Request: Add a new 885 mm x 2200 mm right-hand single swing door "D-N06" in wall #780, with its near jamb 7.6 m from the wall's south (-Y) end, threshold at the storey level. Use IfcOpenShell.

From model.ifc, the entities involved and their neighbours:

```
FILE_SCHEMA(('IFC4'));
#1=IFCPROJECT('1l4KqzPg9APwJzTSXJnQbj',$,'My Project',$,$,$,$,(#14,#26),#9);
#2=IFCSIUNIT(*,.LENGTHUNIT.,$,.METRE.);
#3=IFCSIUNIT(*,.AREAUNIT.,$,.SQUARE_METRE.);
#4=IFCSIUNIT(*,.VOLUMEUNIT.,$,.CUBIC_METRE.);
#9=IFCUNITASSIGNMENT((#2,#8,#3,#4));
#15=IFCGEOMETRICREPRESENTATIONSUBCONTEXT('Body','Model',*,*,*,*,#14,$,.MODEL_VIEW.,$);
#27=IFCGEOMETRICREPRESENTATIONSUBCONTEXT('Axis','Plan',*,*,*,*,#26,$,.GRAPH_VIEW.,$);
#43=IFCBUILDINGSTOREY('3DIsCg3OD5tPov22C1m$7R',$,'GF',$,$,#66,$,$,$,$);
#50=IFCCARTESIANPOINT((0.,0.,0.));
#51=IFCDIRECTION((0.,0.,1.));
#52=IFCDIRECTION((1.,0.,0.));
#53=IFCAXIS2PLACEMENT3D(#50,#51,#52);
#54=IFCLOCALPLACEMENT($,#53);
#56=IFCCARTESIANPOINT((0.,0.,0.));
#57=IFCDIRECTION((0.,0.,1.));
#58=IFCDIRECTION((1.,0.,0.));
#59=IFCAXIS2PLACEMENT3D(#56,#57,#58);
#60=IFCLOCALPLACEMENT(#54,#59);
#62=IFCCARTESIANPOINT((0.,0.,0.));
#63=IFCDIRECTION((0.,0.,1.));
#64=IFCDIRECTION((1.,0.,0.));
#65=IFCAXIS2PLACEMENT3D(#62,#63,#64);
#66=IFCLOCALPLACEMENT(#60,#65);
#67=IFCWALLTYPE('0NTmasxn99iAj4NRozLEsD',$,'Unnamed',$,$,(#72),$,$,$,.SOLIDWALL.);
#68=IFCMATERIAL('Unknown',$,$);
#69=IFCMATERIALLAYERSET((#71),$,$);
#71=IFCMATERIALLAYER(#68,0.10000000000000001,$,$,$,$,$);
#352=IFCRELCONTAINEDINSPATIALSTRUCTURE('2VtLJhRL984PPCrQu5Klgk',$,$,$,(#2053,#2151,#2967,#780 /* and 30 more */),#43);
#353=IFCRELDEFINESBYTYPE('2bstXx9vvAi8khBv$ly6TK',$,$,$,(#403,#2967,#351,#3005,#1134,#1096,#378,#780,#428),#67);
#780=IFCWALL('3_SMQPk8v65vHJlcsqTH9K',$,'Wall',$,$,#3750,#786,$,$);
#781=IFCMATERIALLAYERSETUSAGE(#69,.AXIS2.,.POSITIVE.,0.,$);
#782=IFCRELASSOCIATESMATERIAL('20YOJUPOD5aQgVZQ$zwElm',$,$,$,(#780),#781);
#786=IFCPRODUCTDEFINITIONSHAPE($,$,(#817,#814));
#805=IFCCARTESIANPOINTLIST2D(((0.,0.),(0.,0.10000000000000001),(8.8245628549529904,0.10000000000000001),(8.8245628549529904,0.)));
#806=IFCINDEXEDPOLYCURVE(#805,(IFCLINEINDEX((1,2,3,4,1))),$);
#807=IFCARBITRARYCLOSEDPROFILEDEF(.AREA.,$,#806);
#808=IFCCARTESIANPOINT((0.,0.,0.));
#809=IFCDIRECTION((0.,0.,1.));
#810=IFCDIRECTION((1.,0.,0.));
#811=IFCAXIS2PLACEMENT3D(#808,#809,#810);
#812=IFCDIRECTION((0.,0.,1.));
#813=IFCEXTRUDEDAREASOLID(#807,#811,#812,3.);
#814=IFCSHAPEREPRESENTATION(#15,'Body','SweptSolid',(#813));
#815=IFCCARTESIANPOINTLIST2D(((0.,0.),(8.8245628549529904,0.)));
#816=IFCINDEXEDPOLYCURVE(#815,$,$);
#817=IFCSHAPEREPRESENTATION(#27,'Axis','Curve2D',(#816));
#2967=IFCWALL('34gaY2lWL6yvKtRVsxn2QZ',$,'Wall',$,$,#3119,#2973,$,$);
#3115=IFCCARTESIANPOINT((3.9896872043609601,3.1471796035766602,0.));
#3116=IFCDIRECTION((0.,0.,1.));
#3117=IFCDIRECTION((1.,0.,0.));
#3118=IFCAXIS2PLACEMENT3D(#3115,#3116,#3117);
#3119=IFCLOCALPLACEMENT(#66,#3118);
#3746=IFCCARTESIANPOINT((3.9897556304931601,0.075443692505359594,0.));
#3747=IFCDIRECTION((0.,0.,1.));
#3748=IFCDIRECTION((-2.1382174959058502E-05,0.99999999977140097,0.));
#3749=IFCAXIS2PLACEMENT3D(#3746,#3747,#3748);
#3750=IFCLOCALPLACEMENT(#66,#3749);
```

```python
import numpy as np
import ifcopenshell
import ifcopenshell.api.feature
import ifcopenshell.api.geometry
import ifcopenshell.api.root
import ifcopenshell.api.spatial
import ifcopenshell.geom
import ifcopenshell.util.element
import ifcopenshell.util.placement
import ifcopenshell.util.representation
import ifcopenshell.util.shape
import ifcopenshell.util.unit

model = ifcopenshell.open("model.ifc")
unit_scale = ifcopenshell.util.unit.calculate_unit_scale(model)
settings = ifcopenshell.geom.settings()


def volume(element):
    """Net volume in cubic metres, openings subtracted."""
    shape = ifcopenshell.geom.create_shape(settings, element)
    return ifcopenshell.util.shape.get_volume(shape.geometry)


wall = model.by_guid("3_SMQPk8v65vHJlcsqTH9K")
storey = ifcopenshell.util.element.get_container(wall, ifc_class="IfcBuildingStorey")
context = ifcopenshell.util.representation.get_context(model, "Model", "Body", "MODEL_VIEW")
before = volume(wall)

width, height, from_end, sill = 0.885, 2.2, 7.6, 0.0  # metres

# The wall runs along its own X axis, and the end named is its -X end.
wall_shape = ifcopenshell.geom.create_shape(settings, wall)
x, y, z = ifcopenshell.util.shape.get_vertices(wall_shape.geometry).T
start = x.min() + from_end
face, thickness = float(y.min()), float(y.max() - y.min())
wall_matrix = ifcopenshell.util.placement.get_local_placement(wall.ObjectPlacement)
level = ifcopenshell.util.placement.get_local_placement(storey.ObjectPlacement)[2, 3]


def in_wall(x, y):
    """Placement at x, y metres in the wall's axes, at sill height."""
    matrix = wall_matrix.copy()
    matrix[:, 3] = wall_matrix @ np.array([x / unit_scale, y / unit_scale, 0.0, 1.0])
    matrix[2, 3] = level + sill / unit_scale
    return matrix


# Opening: a box that overshoots both wall faces by 50 mm.
opening = ifcopenshell.api.root.create_entity(model, ifc_class="IfcOpeningElement", predefined_type="OPENING")
box = ifcopenshell.api.geometry.add_wall_representation(
    model, context=context, length=width, height=height, thickness=thickness + 0.1
)
ifcopenshell.api.geometry.assign_representation(model, product=opening, representation=box)
ifcopenshell.api.geometry.edit_object_placement(model, product=opening, matrix=in_wall(start, face - 0.05), is_si=False)
ifcopenshell.api.feature.add_feature(model, feature=opening, element=wall)

door = ifcopenshell.api.root.create_entity(model, ifc_class="IfcDoor", name="D-N06", predefined_type="DOOR")
door.OverallWidth, door.OverallHeight = width / unit_scale, height / unit_scale
door.OperationType = "SINGLE_SWING_RIGHT"
body = ifcopenshell.api.geometry.add_door_representation(
    model,
    context=context,
    overall_width=door.OverallWidth,
    overall_height=door.OverallHeight,
    operation_type="SINGLE_SWING_RIGHT",
    lining_properties={"LiningDepth": thickness / unit_scale, "ThresholdDepth": thickness / unit_scale},
)
ifcopenshell.api.geometry.assign_representation(model, product=door, representation=body)
ifcopenshell.api.spatial.assign_container(model, products=[door], relating_structure=storey)
ifcopenshell.api.feature.add_filling(model, opening=opening, element=door)

# The lining spans the wall, so the door starts at the wall face.
ifcopenshell.api.geometry.edit_object_placement(model, product=door, matrix=in_wall(start, face), is_si=False)

after = volume(wall)

print(f"wall volume {before:.3f} -> {after:.3f} m3")

model.write("model_edited.ifc")
```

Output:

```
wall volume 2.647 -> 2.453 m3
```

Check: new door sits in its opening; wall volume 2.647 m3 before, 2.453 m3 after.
